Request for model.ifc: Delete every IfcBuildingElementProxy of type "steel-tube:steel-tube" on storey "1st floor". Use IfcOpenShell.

First a look at what the model holds.

```python
import ifcopenshell
import ifcopenshell.util.element

model = ifcopenshell.open("model.ifc")
print(model.schema)
storey = next(s for s in model.by_type("IfcBuildingStorey") if s.Name == "1st floor")
proxies = [e for e in ifcopenshell.util.element.get_decomposition(storey) if e.is_a("IfcBuildingElementProxy")]
seen = {}
for e in proxies:
    element_type = ifcopenshell.util.element.get_type(e)
    name = element_type.Name if element_type not in (None, e) else None
    seen[name] = seen.get(name, 0) + 1
for name, count in sorted(seen.items(), key=str):
    print(count, "x", name)
```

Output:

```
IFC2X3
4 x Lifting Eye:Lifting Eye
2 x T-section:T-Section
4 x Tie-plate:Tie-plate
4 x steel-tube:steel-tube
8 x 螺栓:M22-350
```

```python
import ifcopenshell
import ifcopenshell.api.root
import ifcopenshell.util.element

model = ifcopenshell.open("model.ifc")

storey = next(s for s in model.by_type("IfcBuildingStorey") if s.Name == "1st floor")
proxies = [e for e in ifcopenshell.util.element.get_decomposition(storey) if e.is_a("IfcBuildingElementProxy")]
targets = [e for e in proxies if (t := ifcopenshell.util.element.get_type(e)) not in (None, e) and t.Name == "steel-tube:steel-tube"]

for e in targets:
    ifcopenshell.api.root.remove_product(model, product=e)
print(len(targets), "removed")

model.write("model-out.ifc")
```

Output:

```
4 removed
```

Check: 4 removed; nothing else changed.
